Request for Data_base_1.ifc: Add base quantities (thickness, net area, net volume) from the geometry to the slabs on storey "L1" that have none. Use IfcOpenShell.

First a look at what the model holds.

```python
import ifcopenshell
import ifcopenshell.util.element
import ifcopenshell.util.unit

model = ifcopenshell.open("Data_base_1.ifc")
print(model.schema)
for unit_type in ("LENGTHUNIT", "AREAUNIT", "VOLUMEUNIT"):
    print(unit_type, ifcopenshell.util.unit.calculate_unit_scale(model, unit_type))
storey = next(s for s in model.by_type("IfcBuildingStorey") if s.Name == "L1")
slabs = [e for e in ifcopenshell.util.element.get_decomposition(storey) if e.is_a("IfcSlab")]
for e in sorted(slabs, key=lambda e: e.id()):
    print(e.id(), e.is_a(), e.Name, list(ifcopenshell.util.element.get_psets(e, qtos_only=True)), sep=" | ")
```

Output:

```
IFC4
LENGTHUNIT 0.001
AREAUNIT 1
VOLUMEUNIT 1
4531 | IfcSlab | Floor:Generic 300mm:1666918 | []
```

```python
import ifcopenshell
import ifcopenshell.api.pset
import ifcopenshell.geom
import ifcopenshell.util.element
import ifcopenshell.util.shape
import ifcopenshell.util.unit

model = ifcopenshell.open("Data_base_1.ifc")
unit_scale = ifcopenshell.util.unit.calculate_unit_scale(model)
area_scale = ifcopenshell.util.unit.calculate_unit_scale(model, "AREAUNIT")
volume_scale = ifcopenshell.util.unit.calculate_unit_scale(model, "VOLUMEUNIT")
settings = ifcopenshell.geom.settings()

storey = next(s for s in model.by_type("IfcBuildingStorey") if s.Name == "L1")
slabs = [e for e in ifcopenshell.util.element.get_decomposition(storey) if e.is_a("IfcSlab")]

for e in sorted(slabs, key=lambda e: e.id()):
    if ifcopenshell.util.element.get_psets(e, qtos_only=True, should_inherit=False):
        continue
    # Geometry comes back in metres, in the element's own axes.
    shape = ifcopenshell.geom.create_shape(settings, e)
    values = {
        "Width": ifcopenshell.util.shape.get_z(shape.geometry) / unit_scale,
        "NetArea": ifcopenshell.util.shape.get_footprint_area(shape.geometry) / area_scale,
        "NetVolume": ifcopenshell.util.shape.get_volume(shape.geometry) / volume_scale,
    }
    qto = ifcopenshell.api.pset.add_qto(model, product=e, name="Qto_SlabBaseQuantities")
    ifcopenshell.api.pset.edit_qto(model, qto=qto, properties=values)
    print(e.id(), {k: round(v, 3) for k, v in values.items()})

model.write("Data_base_1_updated.ifc")
```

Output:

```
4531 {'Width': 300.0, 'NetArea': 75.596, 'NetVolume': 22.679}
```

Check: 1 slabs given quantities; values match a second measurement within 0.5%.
